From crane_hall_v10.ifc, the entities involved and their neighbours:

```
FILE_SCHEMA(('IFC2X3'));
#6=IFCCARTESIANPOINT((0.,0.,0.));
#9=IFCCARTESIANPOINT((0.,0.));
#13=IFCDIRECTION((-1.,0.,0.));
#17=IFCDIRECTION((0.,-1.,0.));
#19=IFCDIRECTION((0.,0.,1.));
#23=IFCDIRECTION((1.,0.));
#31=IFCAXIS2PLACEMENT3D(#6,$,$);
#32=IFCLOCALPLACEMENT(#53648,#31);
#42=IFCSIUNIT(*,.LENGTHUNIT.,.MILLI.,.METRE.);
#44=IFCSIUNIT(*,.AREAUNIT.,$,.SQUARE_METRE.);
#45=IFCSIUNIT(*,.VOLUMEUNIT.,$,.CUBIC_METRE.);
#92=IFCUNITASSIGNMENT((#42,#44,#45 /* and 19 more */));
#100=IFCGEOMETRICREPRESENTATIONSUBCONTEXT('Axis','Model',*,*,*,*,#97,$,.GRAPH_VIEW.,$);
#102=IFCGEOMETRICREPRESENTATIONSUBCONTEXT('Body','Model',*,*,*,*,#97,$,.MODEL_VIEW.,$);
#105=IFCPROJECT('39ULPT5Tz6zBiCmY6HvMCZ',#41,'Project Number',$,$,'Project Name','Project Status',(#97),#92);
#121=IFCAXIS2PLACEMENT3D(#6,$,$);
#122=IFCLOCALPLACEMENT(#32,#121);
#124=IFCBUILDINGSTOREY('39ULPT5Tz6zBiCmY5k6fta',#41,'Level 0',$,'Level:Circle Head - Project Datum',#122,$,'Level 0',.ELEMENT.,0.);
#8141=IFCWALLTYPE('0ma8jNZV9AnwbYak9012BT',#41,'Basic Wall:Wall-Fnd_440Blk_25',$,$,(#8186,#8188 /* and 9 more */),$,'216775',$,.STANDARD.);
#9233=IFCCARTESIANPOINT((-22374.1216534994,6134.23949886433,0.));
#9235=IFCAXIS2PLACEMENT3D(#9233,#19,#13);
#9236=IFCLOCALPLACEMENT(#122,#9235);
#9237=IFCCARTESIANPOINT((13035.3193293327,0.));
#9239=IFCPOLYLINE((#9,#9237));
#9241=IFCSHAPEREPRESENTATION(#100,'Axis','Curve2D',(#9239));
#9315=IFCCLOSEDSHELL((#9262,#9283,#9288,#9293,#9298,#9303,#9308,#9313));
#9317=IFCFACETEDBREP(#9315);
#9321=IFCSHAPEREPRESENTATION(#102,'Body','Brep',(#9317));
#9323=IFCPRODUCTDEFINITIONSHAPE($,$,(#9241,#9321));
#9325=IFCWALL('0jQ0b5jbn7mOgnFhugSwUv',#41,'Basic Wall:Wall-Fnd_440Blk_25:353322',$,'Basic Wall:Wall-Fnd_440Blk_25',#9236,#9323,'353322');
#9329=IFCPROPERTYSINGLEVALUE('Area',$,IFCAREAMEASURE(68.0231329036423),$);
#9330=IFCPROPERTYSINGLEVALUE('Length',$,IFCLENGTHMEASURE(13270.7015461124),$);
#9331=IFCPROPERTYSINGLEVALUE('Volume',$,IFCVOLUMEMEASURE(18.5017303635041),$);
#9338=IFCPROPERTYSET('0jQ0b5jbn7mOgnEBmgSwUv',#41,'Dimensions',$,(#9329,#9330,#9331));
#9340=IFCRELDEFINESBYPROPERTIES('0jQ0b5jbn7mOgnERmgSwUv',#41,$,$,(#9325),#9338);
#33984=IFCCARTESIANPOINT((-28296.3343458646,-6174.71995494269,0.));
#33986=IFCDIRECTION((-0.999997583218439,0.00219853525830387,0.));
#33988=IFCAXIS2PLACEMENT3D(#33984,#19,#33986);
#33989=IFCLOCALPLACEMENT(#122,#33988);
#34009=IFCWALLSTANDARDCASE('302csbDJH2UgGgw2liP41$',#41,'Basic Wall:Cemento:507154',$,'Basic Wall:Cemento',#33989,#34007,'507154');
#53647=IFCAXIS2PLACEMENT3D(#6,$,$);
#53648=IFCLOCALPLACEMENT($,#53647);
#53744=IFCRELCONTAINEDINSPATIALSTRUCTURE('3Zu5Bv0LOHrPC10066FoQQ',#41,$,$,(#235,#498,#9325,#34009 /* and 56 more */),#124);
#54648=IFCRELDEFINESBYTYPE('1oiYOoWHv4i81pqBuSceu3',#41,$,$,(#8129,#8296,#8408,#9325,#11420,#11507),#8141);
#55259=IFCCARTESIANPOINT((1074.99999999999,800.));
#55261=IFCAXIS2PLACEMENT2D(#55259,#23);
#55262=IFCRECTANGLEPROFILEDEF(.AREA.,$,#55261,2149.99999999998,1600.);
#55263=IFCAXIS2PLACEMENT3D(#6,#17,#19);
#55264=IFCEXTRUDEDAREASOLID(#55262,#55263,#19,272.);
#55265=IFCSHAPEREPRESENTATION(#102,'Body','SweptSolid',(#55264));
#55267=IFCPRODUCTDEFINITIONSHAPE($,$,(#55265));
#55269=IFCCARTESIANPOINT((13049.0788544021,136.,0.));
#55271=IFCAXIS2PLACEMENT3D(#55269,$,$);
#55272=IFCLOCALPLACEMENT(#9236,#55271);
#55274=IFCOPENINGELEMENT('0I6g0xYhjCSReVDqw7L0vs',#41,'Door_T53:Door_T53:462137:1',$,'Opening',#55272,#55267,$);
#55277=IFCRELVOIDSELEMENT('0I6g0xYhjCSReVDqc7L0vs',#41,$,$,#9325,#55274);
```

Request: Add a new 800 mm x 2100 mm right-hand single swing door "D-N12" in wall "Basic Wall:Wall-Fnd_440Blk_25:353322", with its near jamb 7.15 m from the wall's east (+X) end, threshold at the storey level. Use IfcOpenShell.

```python
import numpy as np
import ifcopenshell
import ifcopenshell.api.feature
import ifcopenshell.api.geometry
import ifcopenshell.api.pset
import ifcopenshell.api.root
import ifcopenshell.api.spatial
import ifcopenshell.api.type
import ifcopenshell.geom
import ifcopenshell.util.element
import ifcopenshell.util.placement
import ifcopenshell.util.representation
import ifcopenshell.util.shape
import ifcopenshell.util.unit

model = ifcopenshell.open("crane_hall_v10.ifc")
unit_scale = ifcopenshell.util.unit.calculate_unit_scale(model)
area_scale = ifcopenshell.util.unit.calculate_unit_scale(model, "AREAUNIT")
volume_scale = ifcopenshell.util.unit.calculate_unit_scale(model, "VOLUMEUNIT")
settings = ifcopenshell.geom.settings()


def volume(element):
    """Net volume in cubic metres, openings subtracted."""
    shape = ifcopenshell.geom.create_shape(settings, element)
    return ifcopenshell.util.shape.get_volume(shape.geometry)


wall = model.by_guid("0jQ0b5jbn7mOgnFhugSwUv")
storey = ifcopenshell.util.element.get_container(wall, ifc_class="IfcBuildingStorey")
context = ifcopenshell.util.representation.get_context(model, "Model", "Body", "MODEL_VIEW")
before = volume(wall)

width, height, from_end, sill = 0.8, 2.1, 7.15, 0.0  # metres

# The wall runs along its own X axis, and the end named is its -X end.
wall_shape = ifcopenshell.geom.create_shape(settings, wall)
x, y, z = ifcopenshell.util.shape.get_vertices(wall_shape.geometry).T
start = x.min() + from_end
face, thickness = float(y.min()), float(y.max() - y.min())
wall_matrix = ifcopenshell.util.placement.get_local_placement(wall.ObjectPlacement)
level = ifcopenshell.util.placement.get_local_placement(storey.ObjectPlacement)[2, 3]


def in_wall(x, y):
    """Placement at x, y metres in the wall's axes, at sill height."""
    matrix = wall_matrix.copy()
    matrix[:, 3] = wall_matrix @ np.array([x / unit_scale, y / unit_scale, 0.0, 1.0])
    matrix[2, 3] = level + sill / unit_scale
    return matrix


# Opening: a box that overshoots both wall faces by 50 mm.
opening = ifcopenshell.api.root.create_entity(model, ifc_class="IfcOpeningElement")
box = ifcopenshell.api.geometry.add_wall_representation(
    model, context=context, length=width, height=height, thickness=thickness + 0.1
)
ifcopenshell.api.geometry.assign_representation(model, product=opening, representation=box)
ifcopenshell.api.geometry.edit_object_placement(model, product=opening, matrix=in_wall(start, face - 0.05), is_si=False)
ifcopenshell.api.feature.add_feature(model, feature=opening, element=wall)

door = ifcopenshell.api.root.create_entity(model, ifc_class="IfcDoor", name="D-N12")
door.OverallWidth, door.OverallHeight = width / unit_scale, height / unit_scale
body = ifcopenshell.api.geometry.add_door_representation(
    model,
    context=context,
    overall_width=door.OverallWidth,
    overall_height=door.OverallHeight,
    operation_type="SINGLE_SWING_RIGHT",
    lining_properties={"LiningDepth": thickness / unit_scale, "ThresholdDepth": thickness / unit_scale},
)
ifcopenshell.api.geometry.assign_representation(model, product=door, representation=body)
ifcopenshell.api.spatial.assign_container(model, products=[door], relating_structure=storey)
fills = ifcopenshell.api.feature.add_filling(model, opening=opening, element=door)
fills.OwnerHistory = door.OwnerHistory  # required in IFC2X3

# IFC2X3 keeps the operation on the door style.
style = ifcopenshell.api.root.create_entity(model, ifc_class="IfcDoorStyle", name="D-N12")
style.OperationType, style.ConstructionType = "SINGLE_SWING_RIGHT", "NOTDEFINED"
style.ParameterTakesPrecedence = style.Sizeable = False
ifcopenshell.api.type.assign_type(model, related_objects=[door], relating_type=style)

# The lining spans the wall, so the door starts at the wall face.
ifcopenshell.api.geometry.edit_object_placement(model, product=door, matrix=in_wall(start, face), is_si=False)

after = volume(wall)

# Update the wall's stored quantities.
pset = model.by_id(ifcopenshell.util.element.get_pset(wall, "Dimensions", should_inherit=False)["id"])
ifcopenshell.api.pset.edit_pset(model, pset=pset, properties={
    "Area": model.create_entity("IfcAreaMeasure", after / thickness / area_scale),
    "Volume": model.create_entity("IfcVolumeMeasure", after / volume_scale),
})

print(f"wall volume {before:.3f} -> {after:.3f} m3")

model.write("crane_hall_v10_updated.ifc")
```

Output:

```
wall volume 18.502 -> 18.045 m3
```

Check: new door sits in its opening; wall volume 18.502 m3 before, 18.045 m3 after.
